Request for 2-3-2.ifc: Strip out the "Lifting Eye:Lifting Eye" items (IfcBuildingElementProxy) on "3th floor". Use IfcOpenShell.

First a look at what the model holds.

```python
import ifcopenshell
import ifcopenshell.util.element

model = ifcopenshell.open("2-3-2.ifc")
print(model.schema)
storey = next(s for s in model.by_type("IfcBuildingStorey") if s.Name == "3th floor")
proxies = [e for e in ifcopenshell.util.element.get_decomposition(storey) if e.is_a("IfcBuildingElementProxy")]
seen = {}
for e in proxies:
    element_type = ifcopenshell.util.element.get_type(e)
    name = element_type.Name if element_type not in (None, e) else None
    seen[name] = seen.get(name, 0) + 1
for name, count in sorted(seen.items(), key=str):
    print(count, "x", name)
```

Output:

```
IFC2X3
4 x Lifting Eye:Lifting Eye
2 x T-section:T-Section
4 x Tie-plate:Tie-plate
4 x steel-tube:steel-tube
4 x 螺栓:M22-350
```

```python
import ifcopenshell
import ifcopenshell.api.root
import ifcopenshell.util.element

model = ifcopenshell.open("2-3-2.ifc")

storey = next(s for s in model.by_type("IfcBuildingStorey") if s.Name == "3th floor")
proxies = [e for e in ifcopenshell.util.element.get_decomposition(storey) if e.is_a("IfcBuildingElementProxy")]
targets = [e for e in proxies if (t := ifcopenshell.util.element.get_type(e)) not in (None, e) and t.Name == "Lifting Eye:Lifting Eye"]

for e in targets:
    ifcopenshell.api.root.remove_product(model, product=e)
print(len(targets), "removed")

model.write("2-3-2_edited.ifc")
```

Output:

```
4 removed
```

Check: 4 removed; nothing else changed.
